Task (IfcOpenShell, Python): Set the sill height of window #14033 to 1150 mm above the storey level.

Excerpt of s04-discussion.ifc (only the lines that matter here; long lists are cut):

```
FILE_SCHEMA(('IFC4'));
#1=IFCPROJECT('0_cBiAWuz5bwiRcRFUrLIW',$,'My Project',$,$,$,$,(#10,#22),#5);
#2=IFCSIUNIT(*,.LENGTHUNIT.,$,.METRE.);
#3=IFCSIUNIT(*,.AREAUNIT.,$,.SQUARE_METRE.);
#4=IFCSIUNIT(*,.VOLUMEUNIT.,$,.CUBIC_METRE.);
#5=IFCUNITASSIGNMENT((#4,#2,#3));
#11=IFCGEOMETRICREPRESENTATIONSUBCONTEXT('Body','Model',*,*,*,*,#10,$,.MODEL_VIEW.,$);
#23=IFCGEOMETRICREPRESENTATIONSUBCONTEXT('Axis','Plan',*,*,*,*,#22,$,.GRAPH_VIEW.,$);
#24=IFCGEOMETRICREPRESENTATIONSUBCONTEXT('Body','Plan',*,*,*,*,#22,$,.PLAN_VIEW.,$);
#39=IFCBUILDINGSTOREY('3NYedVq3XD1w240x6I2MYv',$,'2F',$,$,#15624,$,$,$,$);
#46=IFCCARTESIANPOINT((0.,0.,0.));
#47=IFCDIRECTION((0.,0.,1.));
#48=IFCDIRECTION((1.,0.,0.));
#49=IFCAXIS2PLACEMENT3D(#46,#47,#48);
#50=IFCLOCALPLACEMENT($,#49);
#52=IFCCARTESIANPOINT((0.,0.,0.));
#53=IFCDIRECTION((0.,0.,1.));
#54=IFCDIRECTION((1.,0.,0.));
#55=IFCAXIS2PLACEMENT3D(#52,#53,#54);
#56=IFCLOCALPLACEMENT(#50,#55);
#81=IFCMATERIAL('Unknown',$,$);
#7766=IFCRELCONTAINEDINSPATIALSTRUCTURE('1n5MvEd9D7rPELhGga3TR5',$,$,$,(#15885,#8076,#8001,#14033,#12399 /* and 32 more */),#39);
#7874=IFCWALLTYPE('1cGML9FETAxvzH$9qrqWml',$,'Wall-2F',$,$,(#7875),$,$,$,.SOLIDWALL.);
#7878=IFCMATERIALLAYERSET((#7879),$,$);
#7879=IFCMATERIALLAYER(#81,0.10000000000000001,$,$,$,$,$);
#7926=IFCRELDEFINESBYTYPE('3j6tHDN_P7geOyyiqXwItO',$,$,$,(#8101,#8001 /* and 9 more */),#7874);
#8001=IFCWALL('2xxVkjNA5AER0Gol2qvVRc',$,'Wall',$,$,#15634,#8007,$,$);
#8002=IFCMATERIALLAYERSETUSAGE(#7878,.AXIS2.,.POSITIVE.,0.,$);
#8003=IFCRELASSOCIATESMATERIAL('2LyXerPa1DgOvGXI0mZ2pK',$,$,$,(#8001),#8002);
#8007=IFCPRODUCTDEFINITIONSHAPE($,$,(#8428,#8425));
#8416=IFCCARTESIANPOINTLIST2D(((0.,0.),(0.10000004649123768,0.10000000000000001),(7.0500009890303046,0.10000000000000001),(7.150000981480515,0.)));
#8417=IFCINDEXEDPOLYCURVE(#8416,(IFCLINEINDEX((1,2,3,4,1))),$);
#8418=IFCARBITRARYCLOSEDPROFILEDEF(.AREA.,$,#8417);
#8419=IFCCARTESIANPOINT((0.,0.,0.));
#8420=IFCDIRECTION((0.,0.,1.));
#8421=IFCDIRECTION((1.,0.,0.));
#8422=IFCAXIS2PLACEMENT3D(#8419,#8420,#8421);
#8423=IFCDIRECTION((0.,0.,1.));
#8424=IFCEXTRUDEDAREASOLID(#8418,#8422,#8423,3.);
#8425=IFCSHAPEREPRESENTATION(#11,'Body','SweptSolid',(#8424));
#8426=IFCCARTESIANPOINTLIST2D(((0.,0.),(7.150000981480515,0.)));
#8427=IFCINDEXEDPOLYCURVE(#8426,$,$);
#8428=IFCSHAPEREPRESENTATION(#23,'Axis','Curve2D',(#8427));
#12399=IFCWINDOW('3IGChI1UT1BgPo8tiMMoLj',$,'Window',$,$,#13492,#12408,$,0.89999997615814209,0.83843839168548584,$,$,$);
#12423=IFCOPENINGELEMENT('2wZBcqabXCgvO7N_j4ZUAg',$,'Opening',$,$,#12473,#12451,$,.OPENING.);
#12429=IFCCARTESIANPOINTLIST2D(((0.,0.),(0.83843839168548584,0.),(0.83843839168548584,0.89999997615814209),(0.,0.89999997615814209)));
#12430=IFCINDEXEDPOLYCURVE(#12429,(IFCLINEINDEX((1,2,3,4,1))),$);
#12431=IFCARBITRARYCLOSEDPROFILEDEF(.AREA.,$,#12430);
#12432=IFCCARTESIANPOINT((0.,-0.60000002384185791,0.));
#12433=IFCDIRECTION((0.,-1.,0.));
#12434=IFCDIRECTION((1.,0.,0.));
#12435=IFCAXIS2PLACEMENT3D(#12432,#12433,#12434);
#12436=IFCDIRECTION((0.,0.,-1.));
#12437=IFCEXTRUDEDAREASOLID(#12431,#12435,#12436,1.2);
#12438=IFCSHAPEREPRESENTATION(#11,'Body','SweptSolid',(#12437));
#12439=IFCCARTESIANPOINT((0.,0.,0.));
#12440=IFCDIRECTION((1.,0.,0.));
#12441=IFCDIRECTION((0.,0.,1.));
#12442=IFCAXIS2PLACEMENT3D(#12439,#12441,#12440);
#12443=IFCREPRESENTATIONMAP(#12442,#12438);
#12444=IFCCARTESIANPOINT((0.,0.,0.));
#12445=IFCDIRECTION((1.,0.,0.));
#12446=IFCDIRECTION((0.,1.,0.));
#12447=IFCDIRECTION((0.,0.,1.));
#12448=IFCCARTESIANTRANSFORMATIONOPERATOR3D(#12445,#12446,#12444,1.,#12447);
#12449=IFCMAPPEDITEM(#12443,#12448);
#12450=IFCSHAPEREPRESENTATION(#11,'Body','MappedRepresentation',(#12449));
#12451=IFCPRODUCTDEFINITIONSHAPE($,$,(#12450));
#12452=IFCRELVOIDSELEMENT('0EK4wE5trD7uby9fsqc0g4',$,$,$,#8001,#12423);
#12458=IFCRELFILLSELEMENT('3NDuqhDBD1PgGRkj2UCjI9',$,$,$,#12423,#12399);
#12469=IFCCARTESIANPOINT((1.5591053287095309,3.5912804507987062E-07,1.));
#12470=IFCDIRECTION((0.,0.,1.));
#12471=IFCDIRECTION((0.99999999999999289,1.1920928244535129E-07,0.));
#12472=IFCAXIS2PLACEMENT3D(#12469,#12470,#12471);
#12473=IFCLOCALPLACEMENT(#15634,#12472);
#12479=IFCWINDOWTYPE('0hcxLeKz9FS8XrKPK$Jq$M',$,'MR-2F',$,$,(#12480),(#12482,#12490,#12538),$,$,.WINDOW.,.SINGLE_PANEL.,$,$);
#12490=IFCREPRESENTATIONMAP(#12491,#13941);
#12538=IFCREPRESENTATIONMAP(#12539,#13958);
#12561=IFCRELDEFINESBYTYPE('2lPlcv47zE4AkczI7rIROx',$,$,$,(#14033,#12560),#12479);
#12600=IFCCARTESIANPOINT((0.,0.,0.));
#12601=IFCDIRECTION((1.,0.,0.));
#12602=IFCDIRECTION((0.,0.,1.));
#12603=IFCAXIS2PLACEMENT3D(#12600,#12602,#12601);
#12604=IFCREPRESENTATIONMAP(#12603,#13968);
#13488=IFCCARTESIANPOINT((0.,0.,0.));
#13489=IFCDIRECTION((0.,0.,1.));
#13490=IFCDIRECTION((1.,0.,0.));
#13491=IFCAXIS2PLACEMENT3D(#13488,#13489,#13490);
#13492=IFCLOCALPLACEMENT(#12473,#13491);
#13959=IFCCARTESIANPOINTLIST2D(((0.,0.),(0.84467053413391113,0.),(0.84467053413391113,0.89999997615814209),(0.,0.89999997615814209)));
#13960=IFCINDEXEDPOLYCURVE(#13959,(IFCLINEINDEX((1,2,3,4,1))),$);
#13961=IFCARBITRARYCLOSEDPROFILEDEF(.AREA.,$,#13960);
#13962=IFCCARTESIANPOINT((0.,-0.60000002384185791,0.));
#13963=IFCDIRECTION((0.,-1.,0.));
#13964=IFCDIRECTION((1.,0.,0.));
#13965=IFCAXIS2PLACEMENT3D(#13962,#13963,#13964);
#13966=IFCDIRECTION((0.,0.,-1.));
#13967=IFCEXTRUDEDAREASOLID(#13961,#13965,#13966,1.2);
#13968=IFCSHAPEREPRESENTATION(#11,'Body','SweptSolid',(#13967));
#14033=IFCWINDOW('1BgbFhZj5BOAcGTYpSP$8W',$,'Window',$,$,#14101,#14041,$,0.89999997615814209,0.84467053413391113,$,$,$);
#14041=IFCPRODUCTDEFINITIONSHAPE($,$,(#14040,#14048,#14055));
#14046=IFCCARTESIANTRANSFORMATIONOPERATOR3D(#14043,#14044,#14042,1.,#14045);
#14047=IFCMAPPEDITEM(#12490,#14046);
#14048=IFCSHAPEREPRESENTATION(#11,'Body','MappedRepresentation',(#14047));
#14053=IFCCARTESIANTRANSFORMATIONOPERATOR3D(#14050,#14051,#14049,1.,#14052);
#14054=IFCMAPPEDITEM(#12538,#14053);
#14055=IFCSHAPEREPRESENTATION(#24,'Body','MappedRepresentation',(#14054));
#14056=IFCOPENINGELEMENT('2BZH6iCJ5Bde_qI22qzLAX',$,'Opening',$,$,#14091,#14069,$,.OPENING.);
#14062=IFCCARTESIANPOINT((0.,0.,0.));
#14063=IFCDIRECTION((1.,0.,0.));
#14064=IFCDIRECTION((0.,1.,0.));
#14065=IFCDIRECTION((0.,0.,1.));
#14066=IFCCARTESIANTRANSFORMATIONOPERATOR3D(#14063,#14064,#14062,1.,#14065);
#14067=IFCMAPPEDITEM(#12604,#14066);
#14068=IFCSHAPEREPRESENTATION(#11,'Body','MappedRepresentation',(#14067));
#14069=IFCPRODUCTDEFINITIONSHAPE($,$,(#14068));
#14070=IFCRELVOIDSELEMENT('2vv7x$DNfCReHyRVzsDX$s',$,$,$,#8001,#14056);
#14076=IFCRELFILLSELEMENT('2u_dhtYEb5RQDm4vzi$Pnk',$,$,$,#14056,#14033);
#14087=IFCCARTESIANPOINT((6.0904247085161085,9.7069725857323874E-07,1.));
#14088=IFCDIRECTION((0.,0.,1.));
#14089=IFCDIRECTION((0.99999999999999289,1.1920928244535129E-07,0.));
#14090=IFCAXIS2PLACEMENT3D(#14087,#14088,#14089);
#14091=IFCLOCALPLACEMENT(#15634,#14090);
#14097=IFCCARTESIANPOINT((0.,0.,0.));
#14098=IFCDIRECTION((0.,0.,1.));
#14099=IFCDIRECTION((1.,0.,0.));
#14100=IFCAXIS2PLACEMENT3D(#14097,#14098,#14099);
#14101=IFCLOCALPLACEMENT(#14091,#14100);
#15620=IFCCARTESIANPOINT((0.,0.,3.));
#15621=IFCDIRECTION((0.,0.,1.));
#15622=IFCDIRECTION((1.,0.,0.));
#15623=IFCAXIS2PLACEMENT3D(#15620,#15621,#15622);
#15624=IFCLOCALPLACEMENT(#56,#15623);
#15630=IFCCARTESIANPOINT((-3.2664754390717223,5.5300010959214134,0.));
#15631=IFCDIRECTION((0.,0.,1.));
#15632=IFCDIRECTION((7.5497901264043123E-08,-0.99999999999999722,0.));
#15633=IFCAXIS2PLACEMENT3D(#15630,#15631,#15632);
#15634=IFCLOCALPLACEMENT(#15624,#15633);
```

```python
import numpy as np
import ifcopenshell
import ifcopenshell.api.geometry
import ifcopenshell.geom
import ifcopenshell.util.element
import ifcopenshell.util.placement
import ifcopenshell.util.shape
import ifcopenshell.util.unit

model = ifcopenshell.open("s04-discussion.ifc")
unit_scale = ifcopenshell.util.unit.calculate_unit_scale(model)

window = model.by_id(14033)
opening = window.FillsVoids[0].RelatingOpeningElement
storey = ifcopenshell.util.element.get_container(window, ifc_class="IfcBuildingStorey")
level = ifcopenshell.util.placement.get_local_placement(storey.ObjectPlacement)[2, 3]

# The opening's origin need not be at the sill, so measure its lowest point.
shape = ifcopenshell.geom.create_shape(ifcopenshell.geom.settings(), opening)
bottom = ifcopenshell.util.shape.get_shape_bottom_elevation(shape, shape.geometry) / unit_scale
dz = level + 1.15 / unit_scale - bottom

shift = np.array([0.0, 0.0, dz])
# The window is placed relative to its opening, so it follows when the opening moves.
matrix = ifcopenshell.util.placement.get_local_placement(opening.ObjectPlacement)
matrix[:3, 3] += shift
ifcopenshell.api.geometry.edit_object_placement(
    model, product=opening, matrix=matrix, is_si=False, should_transform_children=True
)

print(f"moved by {dz * unit_scale:+.3f} m")

model.write("s04-discussion-out.ifc")
```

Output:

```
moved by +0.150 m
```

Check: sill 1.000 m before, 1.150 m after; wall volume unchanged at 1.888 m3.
